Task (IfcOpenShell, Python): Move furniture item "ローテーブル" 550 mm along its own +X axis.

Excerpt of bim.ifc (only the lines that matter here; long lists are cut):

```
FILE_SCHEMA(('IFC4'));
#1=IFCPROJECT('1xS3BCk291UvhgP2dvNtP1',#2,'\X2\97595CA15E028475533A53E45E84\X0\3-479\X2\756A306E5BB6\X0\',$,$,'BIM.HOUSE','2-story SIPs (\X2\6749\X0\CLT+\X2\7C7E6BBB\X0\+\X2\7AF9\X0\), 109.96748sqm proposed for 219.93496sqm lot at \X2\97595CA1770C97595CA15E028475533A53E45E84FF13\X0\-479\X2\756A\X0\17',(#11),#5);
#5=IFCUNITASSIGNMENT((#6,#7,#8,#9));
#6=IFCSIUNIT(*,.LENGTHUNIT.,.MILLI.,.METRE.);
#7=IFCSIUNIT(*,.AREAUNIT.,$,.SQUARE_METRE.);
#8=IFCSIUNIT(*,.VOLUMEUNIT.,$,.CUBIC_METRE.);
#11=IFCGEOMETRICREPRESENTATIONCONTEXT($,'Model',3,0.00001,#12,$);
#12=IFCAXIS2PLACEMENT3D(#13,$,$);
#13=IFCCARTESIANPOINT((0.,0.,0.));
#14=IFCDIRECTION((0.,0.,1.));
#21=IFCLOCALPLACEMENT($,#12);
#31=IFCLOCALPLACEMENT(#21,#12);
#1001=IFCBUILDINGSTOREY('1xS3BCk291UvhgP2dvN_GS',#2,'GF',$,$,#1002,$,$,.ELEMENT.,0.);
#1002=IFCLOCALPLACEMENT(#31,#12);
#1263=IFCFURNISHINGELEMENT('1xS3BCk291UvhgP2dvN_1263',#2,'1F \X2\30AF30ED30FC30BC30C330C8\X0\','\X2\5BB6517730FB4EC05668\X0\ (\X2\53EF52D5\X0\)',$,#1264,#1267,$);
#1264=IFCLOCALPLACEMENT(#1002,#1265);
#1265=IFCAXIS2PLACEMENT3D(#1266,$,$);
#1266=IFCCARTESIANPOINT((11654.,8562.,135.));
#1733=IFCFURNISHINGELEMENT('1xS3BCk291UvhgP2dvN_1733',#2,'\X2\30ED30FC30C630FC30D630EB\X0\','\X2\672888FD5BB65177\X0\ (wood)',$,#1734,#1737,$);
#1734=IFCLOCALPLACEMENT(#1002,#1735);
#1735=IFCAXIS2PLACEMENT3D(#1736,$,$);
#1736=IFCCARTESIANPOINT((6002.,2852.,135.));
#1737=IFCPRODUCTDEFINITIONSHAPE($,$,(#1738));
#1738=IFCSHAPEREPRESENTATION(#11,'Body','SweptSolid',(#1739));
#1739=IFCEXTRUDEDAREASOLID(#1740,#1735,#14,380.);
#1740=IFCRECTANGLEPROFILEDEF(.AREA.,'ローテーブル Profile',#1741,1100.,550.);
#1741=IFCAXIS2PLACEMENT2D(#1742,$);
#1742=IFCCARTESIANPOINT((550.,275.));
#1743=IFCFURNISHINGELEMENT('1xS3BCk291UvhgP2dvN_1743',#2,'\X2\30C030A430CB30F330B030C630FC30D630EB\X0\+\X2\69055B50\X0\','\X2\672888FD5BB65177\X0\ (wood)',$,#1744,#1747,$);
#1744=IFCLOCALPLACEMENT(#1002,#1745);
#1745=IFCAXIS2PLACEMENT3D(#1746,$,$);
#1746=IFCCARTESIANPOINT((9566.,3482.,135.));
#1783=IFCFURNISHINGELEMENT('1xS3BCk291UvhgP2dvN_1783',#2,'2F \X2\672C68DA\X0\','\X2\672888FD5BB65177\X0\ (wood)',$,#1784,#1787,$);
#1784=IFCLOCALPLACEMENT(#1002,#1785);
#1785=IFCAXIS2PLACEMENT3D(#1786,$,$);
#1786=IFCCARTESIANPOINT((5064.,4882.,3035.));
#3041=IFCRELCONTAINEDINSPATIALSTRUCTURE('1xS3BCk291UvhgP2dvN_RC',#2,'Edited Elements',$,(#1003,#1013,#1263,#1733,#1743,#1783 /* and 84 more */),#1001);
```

```python
import ifcopenshell
import ifcopenshell.api.geometry
import ifcopenshell.util.placement
import ifcopenshell.util.unit

model = ifcopenshell.open("bim.ifc")
unit_scale = ifcopenshell.util.unit.calculate_unit_scale(model)

item = model.by_guid("1xS3BCk291UvhgP2dvN_1733")
matrix = ifcopenshell.util.placement.get_local_placement(item.ObjectPlacement)
matrix[:3, 3] += matrix[:3, 0] * 0.55 / unit_scale
ifcopenshell.api.geometry.edit_object_placement(model, product=item, matrix=matrix, is_si=False)

print(ifcopenshell.util.placement.get_local_placement(item.ObjectPlacement).round(3) + 0.0)

model.write("bim_v2.ifc")
```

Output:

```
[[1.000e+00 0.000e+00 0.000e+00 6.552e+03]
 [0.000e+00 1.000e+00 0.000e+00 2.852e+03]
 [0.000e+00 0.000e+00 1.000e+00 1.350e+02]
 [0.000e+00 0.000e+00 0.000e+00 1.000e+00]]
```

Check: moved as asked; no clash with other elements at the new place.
